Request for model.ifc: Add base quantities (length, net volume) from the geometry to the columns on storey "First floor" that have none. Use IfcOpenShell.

First a look at what the model holds.

```python
import ifcopenshell
import ifcopenshell.util.element
import ifcopenshell.util.unit

model = ifcopenshell.open("model.ifc")
print(model.schema)
for unit_type in ("LENGTHUNIT", "AREAUNIT", "VOLUMEUNIT"):
    print(unit_type, ifcopenshell.util.unit.calculate_unit_scale(model, unit_type))
storey = next(s for s in model.by_type("IfcBuildingStorey") if s.Name == "First floor")
columns = [e for e in ifcopenshell.util.element.get_decomposition(storey) if e.is_a("IfcColumn")]
for e in sorted(columns, key=lambda e: e.id()):
    print(e.id(), e.is_a(), e.Name, list(ifcopenshell.util.element.get_psets(e, qtos_only=True)), sep=" | ")
```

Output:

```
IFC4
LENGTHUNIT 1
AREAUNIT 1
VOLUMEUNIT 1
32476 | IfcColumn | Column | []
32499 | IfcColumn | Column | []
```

```python
import ifcopenshell
import ifcopenshell.api.pset
import ifcopenshell.geom
import ifcopenshell.util.element
import ifcopenshell.util.shape
import ifcopenshell.util.unit

model = ifcopenshell.open("model.ifc")
unit_scale = ifcopenshell.util.unit.calculate_unit_scale(model)
volume_scale = ifcopenshell.util.unit.calculate_unit_scale(model, "VOLUMEUNIT")
settings = ifcopenshell.geom.settings()

storey = next(s for s in model.by_type("IfcBuildingStorey") if s.Name == "First floor")
columns = [e for e in ifcopenshell.util.element.get_decomposition(storey) if e.is_a("IfcColumn")]

for e in sorted(columns, key=lambda e: e.id()):
    if ifcopenshell.util.element.get_psets(e, qtos_only=True, should_inherit=False):
        continue
    # Geometry comes back in metres, in the element's own axes.
    shape = ifcopenshell.geom.create_shape(settings, e)
    values = {
        "Length": ifcopenshell.util.shape.get_z(shape.geometry) / unit_scale,
        "NetVolume": ifcopenshell.util.shape.get_volume(shape.geometry) / volume_scale,
    }
    qto = ifcopenshell.api.pset.add_qto(model, product=e, name="Qto_ColumnBaseQuantities")
    ifcopenshell.api.pset.edit_qto(model, qto=qto, properties=values)
    print(e.id(), {k: round(v, 3) for k, v in values.items()})

model.write("model_edited.ifc")
```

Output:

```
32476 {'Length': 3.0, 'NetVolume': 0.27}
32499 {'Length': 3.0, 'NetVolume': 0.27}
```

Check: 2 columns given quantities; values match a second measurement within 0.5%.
